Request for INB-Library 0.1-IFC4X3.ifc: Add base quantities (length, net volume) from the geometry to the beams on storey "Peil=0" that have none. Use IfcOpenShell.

First a look at what the model holds.

```python
import ifcopenshell
import ifcopenshell.util.element
import ifcopenshell.util.unit

model = ifcopenshell.open("INB-Library 0.1-IFC4X3.ifc")
print(model.schema)
for unit_type in ("LENGTHUNIT", "AREAUNIT", "VOLUMEUNIT"):
    print(unit_type, ifcopenshell.util.unit.calculate_unit_scale(model, unit_type))
storey = next(s for s in model.by_type("IfcBuildingStorey") if s.Name == "Peil=0")
beams = [e for e in ifcopenshell.util.element.get_decomposition(storey) if e.is_a("IfcBeam")]
for e in sorted(beams, key=lambda e: e.id()):
    print(e.id(), e.is_a(), e.Name, list(ifcopenshell.util.element.get_psets(e, qtos_only=True)), sep=" | ")
```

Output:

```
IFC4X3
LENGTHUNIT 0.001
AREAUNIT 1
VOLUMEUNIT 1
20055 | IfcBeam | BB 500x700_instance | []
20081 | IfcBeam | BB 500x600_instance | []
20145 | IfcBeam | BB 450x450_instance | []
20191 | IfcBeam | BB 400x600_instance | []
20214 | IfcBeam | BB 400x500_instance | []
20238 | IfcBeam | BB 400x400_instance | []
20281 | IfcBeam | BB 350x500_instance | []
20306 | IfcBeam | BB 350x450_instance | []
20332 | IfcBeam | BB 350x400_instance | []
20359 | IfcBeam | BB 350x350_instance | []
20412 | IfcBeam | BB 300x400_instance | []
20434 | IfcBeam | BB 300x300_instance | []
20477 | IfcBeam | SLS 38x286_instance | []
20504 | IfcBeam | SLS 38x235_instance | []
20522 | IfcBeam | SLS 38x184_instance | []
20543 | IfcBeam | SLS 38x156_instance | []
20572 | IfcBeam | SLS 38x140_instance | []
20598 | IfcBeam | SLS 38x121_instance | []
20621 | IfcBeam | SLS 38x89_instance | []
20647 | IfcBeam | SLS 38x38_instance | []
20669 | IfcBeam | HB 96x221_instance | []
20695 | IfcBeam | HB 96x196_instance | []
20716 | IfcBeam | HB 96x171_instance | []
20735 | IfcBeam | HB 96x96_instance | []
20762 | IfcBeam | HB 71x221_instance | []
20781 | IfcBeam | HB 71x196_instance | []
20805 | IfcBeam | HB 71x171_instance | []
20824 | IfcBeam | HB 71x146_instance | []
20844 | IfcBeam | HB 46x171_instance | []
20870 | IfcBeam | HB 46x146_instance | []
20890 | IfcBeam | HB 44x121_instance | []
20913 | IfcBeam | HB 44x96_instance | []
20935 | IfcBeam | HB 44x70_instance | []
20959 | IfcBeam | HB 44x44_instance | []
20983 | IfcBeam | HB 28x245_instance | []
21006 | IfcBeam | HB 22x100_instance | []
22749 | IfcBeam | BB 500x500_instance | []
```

```python
import ifcopenshell
import ifcopenshell.api.pset
import ifcopenshell.geom
import ifcopenshell.util.element
import ifcopenshell.util.shape
import ifcopenshell.util.unit

model = ifcopenshell.open("INB-Library 0.1-IFC4X3.ifc")
unit_scale = ifcopenshell.util.unit.calculate_unit_scale(model)
volume_scale = ifcopenshell.util.unit.calculate_unit_scale(model, "VOLUMEUNIT")
settings = ifcopenshell.geom.settings()

storey = next(s for s in model.by_type("IfcBuildingStorey") if s.Name == "Peil=0")
beams = [e for e in ifcopenshell.util.element.get_decomposition(storey) if e.is_a("IfcBeam")]

for e in sorted(beams, key=lambda e: e.id()):
    if ifcopenshell.util.element.get_psets(e, qtos_only=True, should_inherit=False):
        continue
    # Geometry comes back in metres, in the element's own axes.
    shape = ifcopenshell.geom.create_shape(settings, e)
    values = {
        "Length": ifcopenshell.util.shape.get_max_xyz(shape.geometry) / unit_scale,
        "NetVolume": ifcopenshell.util.shape.get_volume(shape.geometry) / volume_scale,
    }
    qto = ifcopenshell.api.pset.add_qto(model, product=e, name="Qto_BeamBaseQuantities")
    ifcopenshell.api.pset.edit_qto(model, qto=qto, properties=values)
    print(e.id(), {k: round(v, 3) for k, v in values.items()})

model.write("INB-Library 0.1-IFC4X3_rev.ifc")
```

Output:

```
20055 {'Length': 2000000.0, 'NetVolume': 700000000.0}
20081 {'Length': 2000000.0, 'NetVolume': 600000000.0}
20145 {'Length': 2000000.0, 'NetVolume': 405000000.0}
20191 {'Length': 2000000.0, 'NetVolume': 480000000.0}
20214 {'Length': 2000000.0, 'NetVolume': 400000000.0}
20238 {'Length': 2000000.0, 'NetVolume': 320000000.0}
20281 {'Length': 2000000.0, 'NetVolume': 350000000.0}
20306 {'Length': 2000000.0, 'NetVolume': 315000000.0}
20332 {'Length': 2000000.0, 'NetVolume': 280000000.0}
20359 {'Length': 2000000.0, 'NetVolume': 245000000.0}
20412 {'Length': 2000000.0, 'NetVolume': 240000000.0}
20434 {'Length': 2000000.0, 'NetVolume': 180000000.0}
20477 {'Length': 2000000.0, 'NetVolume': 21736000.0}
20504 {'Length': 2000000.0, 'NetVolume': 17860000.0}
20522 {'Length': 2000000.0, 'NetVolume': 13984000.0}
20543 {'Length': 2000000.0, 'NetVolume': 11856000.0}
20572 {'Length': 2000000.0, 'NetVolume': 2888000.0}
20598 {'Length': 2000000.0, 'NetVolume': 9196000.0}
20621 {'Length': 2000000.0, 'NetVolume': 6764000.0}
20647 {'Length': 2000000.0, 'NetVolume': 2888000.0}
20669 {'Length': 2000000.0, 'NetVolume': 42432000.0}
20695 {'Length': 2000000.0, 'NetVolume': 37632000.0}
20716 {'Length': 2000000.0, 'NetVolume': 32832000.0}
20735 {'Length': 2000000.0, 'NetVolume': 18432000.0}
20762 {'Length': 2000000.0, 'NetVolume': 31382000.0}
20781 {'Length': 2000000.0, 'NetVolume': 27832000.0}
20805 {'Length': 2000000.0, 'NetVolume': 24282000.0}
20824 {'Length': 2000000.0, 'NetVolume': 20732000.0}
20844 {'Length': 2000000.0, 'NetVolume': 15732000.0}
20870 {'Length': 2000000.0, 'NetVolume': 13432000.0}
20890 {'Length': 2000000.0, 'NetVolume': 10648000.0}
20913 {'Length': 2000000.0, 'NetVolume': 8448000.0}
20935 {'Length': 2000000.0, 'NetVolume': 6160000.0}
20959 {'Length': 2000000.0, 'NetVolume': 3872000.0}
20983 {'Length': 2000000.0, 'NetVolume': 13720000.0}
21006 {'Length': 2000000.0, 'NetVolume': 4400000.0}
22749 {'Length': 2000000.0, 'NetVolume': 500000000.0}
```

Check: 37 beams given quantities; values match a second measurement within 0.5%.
